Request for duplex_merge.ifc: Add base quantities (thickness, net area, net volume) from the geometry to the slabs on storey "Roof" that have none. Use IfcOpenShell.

First a look at what the model holds.

```python
import ifcopenshell
import ifcopenshell.util.element
import ifcopenshell.util.unit

model = ifcopenshell.open("duplex_merge.ifc")
print(model.schema)
for unit_type in ("LENGTHUNIT", "AREAUNIT", "VOLUMEUNIT"):
    print(unit_type, ifcopenshell.util.unit.calculate_unit_scale(model, unit_type))
storey = next(s for s in model.by_type("IfcBuildingStorey") if s.Name == "Roof")
slabs = [e for e in ifcopenshell.util.element.get_decomposition(storey) if e.is_a("IfcSlab")]
for e in sorted(slabs, key=lambda e: e.id()):
    print(e.id(), e.is_a(), e.Name, list(ifcopenshell.util.element.get_psets(e, qtos_only=True)), sep=" | ")
```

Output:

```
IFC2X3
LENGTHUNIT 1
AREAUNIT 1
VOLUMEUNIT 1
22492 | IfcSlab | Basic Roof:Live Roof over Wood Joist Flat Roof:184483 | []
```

```python
import ifcopenshell
import ifcopenshell.api.pset
import ifcopenshell.geom
import ifcopenshell.util.element
import ifcopenshell.util.shape
import ifcopenshell.util.unit

model = ifcopenshell.open("duplex_merge.ifc")
unit_scale = ifcopenshell.util.unit.calculate_unit_scale(model)
area_scale = ifcopenshell.util.unit.calculate_unit_scale(model, "AREAUNIT")
volume_scale = ifcopenshell.util.unit.calculate_unit_scale(model, "VOLUMEUNIT")
settings = ifcopenshell.geom.settings()

storey = next(s for s in model.by_type("IfcBuildingStorey") if s.Name == "Roof")
slabs = [e for e in ifcopenshell.util.element.get_decomposition(storey) if e.is_a("IfcSlab")]

for e in sorted(slabs, key=lambda e: e.id()):
    if ifcopenshell.util.element.get_psets(e, qtos_only=True, should_inherit=False):
        continue
    # Geometry comes back in metres, in the element's own axes.
    shape = ifcopenshell.geom.create_shape(settings, e)
    values = {
        "Width": ifcopenshell.util.shape.get_z(shape.geometry) / unit_scale,
        "NetArea": ifcopenshell.util.shape.get_footprint_area(shape.geometry) / area_scale,
        "NetVolume": ifcopenshell.util.shape.get_volume(shape.geometry) / volume_scale,
    }
    qto = ifcopenshell.api.pset.add_qto(model, product=e, name="BaseQuantities")
    ifcopenshell.api.pset.edit_qto(model, qto=qto, properties=values)
    print(e.id(), {k: round(v, 3) for k, v in values.items()})

model.write("duplex_merge-out.ifc")
```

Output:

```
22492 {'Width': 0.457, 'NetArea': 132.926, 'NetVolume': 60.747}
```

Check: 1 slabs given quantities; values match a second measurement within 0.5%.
